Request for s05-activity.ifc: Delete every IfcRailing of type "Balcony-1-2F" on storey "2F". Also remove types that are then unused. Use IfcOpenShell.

First a look at what the model holds.

```python
import ifcopenshell
import ifcopenshell.util.element

model = ifcopenshell.open("s05-activity.ifc")
print(model.schema)
storey = next(s for s in model.by_type("IfcBuildingStorey") if s.Name == "2F")
railings = [e for e in ifcopenshell.util.element.get_decomposition(storey) if e.is_a("IfcRailing")]
seen = {}
for e in railings:
    element_type = ifcopenshell.util.element.get_type(e)
    name = element_type.Name if element_type not in (None, e) else None
    seen[name] = seen.get(name, 0) + 1
for name, count in sorted(seen.items(), key=str):
    print(count, "x", name)
```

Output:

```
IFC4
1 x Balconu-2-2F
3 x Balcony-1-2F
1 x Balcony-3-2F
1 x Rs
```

```python
import ifcopenshell
import ifcopenshell.api.root
import ifcopenshell.util.element

model = ifcopenshell.open("s05-activity.ifc")

storey = next(s for s in model.by_type("IfcBuildingStorey") if s.Name == "2F")
railings = [e for e in ifcopenshell.util.element.get_decomposition(storey) if e.is_a("IfcRailing")]
targets = [e for e in railings if (t := ifcopenshell.util.element.get_type(e)) not in (None, e) and t.Name == "Balcony-1-2F"]
types = {ifcopenshell.util.element.get_type(e) for e in targets} - {None, *targets}

for e in targets:
    ifcopenshell.api.root.remove_product(model, product=e)
print(len(targets), "removed")

unused = [t for t in types if not ifcopenshell.util.element.get_types(t)]
for t in unused:
    ifcopenshell.api.root.remove_product(model, product=t)
print(len(unused), "unused types removed")

model.write("s05-activity_v2.ifc")
```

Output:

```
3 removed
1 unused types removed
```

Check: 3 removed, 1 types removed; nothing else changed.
